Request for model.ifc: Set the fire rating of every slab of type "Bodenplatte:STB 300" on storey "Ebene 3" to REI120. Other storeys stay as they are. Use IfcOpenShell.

First a look at what the model holds.

```python
import ifcopenshell
import ifcopenshell.util.element

model = ifcopenshell.open("model.ifc")
print(model.schema)
storey = next(s for s in model.by_type("IfcBuildingStorey") if s.Name == "Ebene 3")
slabs = [e for e in ifcopenshell.util.element.get_decomposition(storey) if e.is_a("IfcSlab")]
seen = {}
for e in slabs:
    element_type = ifcopenshell.util.element.get_type(e)
    key = (element_type.Name if element_type != e and element_type else None, ifcopenshell.util.element.get_pset(e, "Pset_SlabCommon", "FireRating"))
    seen[key] = seen.get(key, 0) + 1
for (name, value), count in sorted(seen.items(), key=str):
    print(count, "x", name, "|", value)
```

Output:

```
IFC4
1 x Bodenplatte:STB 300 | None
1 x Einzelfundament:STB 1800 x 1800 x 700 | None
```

```python
import ifcopenshell
import ifcopenshell.api.pset
import ifcopenshell.util.element

model = ifcopenshell.open("model.ifc")

storey = next(s for s in model.by_type("IfcBuildingStorey") if s.Name == "Ebene 3")
slabs = [e for e in ifcopenshell.util.element.get_decomposition(storey) if e.is_a("IfcSlab")]

count = 0
for e in slabs:
    element_type = ifcopenshell.util.element.get_type(e)
    if element_type in (None, e) or element_type.Name != "Bodenplatte:STB 300":
        continue
    # add_pset returns the element's existing set when there is one.
    pset = ifcopenshell.api.pset.add_pset(model, product=e, name="Pset_SlabCommon")
    ifcopenshell.api.pset.edit_pset(model, pset=pset, properties={"FireRating": "REI120"})
    count += 1

print(count, "slabs updated")

model.write("model_edited.ifc")
```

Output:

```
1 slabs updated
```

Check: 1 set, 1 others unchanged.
